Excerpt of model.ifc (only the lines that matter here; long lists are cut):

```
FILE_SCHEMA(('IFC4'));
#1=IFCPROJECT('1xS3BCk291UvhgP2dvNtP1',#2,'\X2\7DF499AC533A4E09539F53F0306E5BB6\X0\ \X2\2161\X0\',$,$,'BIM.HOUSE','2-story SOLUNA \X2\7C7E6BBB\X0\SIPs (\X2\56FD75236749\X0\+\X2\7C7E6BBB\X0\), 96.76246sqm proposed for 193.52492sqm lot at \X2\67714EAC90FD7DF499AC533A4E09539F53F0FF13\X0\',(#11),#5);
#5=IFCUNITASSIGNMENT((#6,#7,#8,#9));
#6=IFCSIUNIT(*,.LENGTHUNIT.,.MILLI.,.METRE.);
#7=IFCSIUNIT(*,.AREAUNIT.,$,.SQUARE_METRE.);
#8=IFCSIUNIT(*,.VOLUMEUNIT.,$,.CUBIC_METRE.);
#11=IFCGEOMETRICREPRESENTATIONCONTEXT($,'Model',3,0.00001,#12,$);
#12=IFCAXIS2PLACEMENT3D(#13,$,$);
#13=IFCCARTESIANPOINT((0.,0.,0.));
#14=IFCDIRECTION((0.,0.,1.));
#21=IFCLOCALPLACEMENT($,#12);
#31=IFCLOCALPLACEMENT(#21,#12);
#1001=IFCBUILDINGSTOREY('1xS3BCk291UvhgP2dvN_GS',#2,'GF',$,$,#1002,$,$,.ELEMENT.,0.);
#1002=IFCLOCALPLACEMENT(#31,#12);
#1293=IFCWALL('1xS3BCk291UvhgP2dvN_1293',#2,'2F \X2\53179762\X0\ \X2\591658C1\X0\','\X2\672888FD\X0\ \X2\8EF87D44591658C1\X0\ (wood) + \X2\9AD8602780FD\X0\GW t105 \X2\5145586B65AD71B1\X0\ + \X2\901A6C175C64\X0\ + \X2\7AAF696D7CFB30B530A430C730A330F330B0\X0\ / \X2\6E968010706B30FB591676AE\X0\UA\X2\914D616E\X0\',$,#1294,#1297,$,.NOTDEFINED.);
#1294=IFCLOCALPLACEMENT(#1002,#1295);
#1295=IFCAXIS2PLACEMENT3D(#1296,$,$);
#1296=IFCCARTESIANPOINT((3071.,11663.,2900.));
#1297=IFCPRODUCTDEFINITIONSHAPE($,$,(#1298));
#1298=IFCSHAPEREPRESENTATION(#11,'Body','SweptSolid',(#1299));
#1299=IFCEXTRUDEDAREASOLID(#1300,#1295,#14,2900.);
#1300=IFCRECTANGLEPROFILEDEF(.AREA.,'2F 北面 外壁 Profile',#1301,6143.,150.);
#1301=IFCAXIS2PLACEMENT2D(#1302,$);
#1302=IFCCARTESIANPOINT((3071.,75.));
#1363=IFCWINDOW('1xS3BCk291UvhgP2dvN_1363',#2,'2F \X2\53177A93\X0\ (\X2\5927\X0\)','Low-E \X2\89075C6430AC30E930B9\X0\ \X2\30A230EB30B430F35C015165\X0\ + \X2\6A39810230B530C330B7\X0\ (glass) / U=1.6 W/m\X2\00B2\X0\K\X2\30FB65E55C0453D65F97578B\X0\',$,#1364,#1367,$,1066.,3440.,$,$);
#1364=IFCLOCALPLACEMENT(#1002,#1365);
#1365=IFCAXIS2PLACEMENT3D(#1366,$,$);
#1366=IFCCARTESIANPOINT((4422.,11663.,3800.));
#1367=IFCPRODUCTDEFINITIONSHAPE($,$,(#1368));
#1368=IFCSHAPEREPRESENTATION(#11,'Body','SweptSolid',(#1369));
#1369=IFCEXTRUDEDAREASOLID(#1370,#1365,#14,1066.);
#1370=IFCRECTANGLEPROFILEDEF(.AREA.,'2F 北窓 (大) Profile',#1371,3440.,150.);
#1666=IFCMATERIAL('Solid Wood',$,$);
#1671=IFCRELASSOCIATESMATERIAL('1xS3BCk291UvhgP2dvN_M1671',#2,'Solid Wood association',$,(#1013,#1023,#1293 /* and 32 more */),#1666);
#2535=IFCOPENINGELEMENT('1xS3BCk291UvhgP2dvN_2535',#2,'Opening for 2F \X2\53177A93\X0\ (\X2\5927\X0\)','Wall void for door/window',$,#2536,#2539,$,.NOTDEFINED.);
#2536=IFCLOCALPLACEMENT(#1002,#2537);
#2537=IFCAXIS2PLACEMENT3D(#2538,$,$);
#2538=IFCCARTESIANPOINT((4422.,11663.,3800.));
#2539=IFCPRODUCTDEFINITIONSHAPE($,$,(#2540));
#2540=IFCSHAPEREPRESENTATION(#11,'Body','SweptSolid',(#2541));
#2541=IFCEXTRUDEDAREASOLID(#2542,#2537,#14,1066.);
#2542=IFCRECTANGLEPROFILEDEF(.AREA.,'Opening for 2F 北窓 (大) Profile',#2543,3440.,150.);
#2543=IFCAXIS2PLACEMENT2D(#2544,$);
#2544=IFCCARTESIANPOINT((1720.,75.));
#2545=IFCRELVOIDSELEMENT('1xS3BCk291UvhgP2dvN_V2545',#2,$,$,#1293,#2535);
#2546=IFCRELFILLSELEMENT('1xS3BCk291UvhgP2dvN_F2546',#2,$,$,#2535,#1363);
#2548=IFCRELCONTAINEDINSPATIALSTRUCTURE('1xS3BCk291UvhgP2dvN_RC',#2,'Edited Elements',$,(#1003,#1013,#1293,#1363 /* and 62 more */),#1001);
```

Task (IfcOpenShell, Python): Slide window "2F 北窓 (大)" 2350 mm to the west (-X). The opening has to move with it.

```python
import ifcopenshell
import ifcopenshell.api.geometry
import ifcopenshell.util.placement

model = ifcopenshell.open("model.ifc")

window = model.by_guid("1xS3BCk291UvhgP2dvN_1363")
opening = window.FillsVoids[0].RelatingOpeningElement
wall = opening.VoidsElements[0].RelatingBuildingElement

wall_matrix = ifcopenshell.util.placement.get_local_placement(wall.ObjectPlacement)
shift = wall_matrix[:3, 0] * -2350.0
before = ifcopenshell.util.placement.get_local_placement(window.ObjectPlacement)[:3, 3].copy()

# The window is not placed relative to its opening, so move both.
for product in (opening, window):
    matrix = ifcopenshell.util.placement.get_local_placement(product.ObjectPlacement)
    matrix[:3, 3] += shift
    ifcopenshell.api.geometry.edit_object_placement(model, product=product, matrix=matrix, is_si=False)

after = ifcopenshell.util.placement.get_local_placement(window.ObjectPlacement)[:3, 3]
print("window moved by", (after - before).round(3) + 0.0)

model.write("model-out.ifc")
```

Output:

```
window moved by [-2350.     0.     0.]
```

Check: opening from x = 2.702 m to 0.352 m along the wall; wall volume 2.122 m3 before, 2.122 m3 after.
